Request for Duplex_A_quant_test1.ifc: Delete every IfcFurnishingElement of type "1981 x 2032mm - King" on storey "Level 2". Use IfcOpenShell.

First a look at what the model holds.

```python
import ifcopenshell
import ifcopenshell.util.element

model = ifcopenshell.open("Duplex_A_quant_test1.ifc")
print(model.schema)
storey = next(s for s in model.by_type("IfcBuildingStorey") if s.Name == "Level 2")
furniture = [e for e in ifcopenshell.util.element.get_decomposition(storey) if e.is_a("IfcFurnishingElement")]
seen = {}
for e in furniture:
    element_type = ifcopenshell.util.element.get_type(e)
    name = element_type.Name if element_type not in (None, e) else None
    seen[name] = seen.get(name, 0) + 1
for name, count in sorted(seen.items(), key=str):
    print(count, "x", name)
```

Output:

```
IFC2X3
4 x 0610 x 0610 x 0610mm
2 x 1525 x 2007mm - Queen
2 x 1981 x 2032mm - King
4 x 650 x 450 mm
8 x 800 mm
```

```python
import ifcopenshell
import ifcopenshell.api.root
import ifcopenshell.util.element

model = ifcopenshell.open("Duplex_A_quant_test1.ifc")

storey = next(s for s in model.by_type("IfcBuildingStorey") if s.Name == "Level 2")
furniture = [e for e in ifcopenshell.util.element.get_decomposition(storey) if e.is_a("IfcFurnishingElement")]
targets = [e for e in furniture if (t := ifcopenshell.util.element.get_type(e)) not in (None, e) and t.Name == "1981 x 2032mm - King"]

for e in targets:
    ifcopenshell.api.root.remove_product(model, product=e)
print(len(targets), "removed")

model.write("Duplex_A_quant_test1-out.ifc")
```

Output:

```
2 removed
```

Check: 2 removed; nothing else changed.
